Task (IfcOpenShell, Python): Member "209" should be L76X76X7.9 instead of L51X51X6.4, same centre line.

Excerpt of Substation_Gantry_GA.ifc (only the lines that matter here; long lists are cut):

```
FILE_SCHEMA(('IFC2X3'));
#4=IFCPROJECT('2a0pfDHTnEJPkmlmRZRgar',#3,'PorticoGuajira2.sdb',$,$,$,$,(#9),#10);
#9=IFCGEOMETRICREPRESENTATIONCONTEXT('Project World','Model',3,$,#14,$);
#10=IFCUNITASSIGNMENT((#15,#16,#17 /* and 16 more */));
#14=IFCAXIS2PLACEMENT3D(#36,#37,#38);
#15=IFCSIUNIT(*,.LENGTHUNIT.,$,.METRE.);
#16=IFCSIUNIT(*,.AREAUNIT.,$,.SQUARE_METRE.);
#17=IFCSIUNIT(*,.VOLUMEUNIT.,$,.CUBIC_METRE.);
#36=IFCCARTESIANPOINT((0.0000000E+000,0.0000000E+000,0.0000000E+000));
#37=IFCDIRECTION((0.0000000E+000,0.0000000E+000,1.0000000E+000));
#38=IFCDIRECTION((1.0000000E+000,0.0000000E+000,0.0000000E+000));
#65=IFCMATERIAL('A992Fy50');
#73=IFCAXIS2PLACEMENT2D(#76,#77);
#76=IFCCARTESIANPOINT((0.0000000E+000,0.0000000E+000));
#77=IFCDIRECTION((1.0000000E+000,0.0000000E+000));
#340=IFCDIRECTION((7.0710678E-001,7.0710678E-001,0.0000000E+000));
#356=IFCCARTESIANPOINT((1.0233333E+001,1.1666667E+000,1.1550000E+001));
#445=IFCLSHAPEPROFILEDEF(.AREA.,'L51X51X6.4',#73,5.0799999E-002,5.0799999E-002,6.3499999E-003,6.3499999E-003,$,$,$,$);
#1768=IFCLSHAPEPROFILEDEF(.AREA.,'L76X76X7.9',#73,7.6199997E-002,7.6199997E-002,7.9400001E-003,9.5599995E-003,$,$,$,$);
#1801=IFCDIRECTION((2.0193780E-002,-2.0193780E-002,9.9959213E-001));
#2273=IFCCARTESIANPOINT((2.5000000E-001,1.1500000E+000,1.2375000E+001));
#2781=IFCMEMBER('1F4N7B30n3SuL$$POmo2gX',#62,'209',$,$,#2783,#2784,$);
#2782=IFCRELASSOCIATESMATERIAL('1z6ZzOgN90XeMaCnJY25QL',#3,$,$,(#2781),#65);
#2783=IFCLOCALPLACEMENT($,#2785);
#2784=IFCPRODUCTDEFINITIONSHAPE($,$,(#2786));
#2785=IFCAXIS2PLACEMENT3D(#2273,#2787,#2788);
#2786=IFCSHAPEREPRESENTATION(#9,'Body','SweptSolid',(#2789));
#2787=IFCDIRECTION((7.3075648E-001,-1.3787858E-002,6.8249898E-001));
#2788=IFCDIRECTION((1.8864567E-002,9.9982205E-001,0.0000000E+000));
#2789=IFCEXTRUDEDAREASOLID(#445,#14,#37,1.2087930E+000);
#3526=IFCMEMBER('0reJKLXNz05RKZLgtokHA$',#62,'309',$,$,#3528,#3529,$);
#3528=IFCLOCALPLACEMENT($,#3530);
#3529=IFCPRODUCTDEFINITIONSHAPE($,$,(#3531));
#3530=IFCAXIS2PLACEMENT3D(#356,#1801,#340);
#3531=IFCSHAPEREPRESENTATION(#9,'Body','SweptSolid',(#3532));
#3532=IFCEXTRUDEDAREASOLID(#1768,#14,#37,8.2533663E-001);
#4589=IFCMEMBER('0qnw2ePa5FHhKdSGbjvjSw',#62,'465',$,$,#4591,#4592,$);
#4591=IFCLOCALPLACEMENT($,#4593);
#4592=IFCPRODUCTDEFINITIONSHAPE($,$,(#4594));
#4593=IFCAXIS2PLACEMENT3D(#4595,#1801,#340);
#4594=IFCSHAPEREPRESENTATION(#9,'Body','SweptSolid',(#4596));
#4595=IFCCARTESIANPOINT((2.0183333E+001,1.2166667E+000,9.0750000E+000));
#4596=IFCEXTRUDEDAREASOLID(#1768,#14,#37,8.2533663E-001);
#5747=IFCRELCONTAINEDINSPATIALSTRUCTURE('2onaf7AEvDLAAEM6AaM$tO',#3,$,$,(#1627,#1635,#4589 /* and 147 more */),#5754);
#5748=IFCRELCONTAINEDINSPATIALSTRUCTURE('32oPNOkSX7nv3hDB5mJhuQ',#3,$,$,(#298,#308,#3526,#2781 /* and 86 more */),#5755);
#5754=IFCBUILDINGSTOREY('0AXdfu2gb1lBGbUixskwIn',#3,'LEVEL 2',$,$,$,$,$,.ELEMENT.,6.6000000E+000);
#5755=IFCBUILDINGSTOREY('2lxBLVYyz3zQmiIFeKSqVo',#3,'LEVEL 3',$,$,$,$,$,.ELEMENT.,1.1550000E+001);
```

```python
import ifcopenshell
import ifcopenshell.util.element

model = ifcopenshell.open("Substation_Gantry_GA.ifc")

member = model.by_id(2781)
source = next(p for p in model.by_type("IfcLShapeProfileDef") if p.ProfileName == "L76X76X7.9")

body = next(r for r in member.Representation.Representations if r.RepresentationIdentifier == "Body")
solid = body.Items[0]
old_profile = solid.SweptArea

# Copy the section's sizes but keep this member's own profile position.
profile = ifcopenshell.util.element.copy(model, source)
profile.Position = old_profile.Position
solid.SweptArea = profile
if not model.get_total_inverses(old_profile):
    ifcopenshell.util.element.remove_deep2(model, old_profile)

print(solid.SweptArea)

model.write("Substation_Gantry_GA_v2.ifc")
```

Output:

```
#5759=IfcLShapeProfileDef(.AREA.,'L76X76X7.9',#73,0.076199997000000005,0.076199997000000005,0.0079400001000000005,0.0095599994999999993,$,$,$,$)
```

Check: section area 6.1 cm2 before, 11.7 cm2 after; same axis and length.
